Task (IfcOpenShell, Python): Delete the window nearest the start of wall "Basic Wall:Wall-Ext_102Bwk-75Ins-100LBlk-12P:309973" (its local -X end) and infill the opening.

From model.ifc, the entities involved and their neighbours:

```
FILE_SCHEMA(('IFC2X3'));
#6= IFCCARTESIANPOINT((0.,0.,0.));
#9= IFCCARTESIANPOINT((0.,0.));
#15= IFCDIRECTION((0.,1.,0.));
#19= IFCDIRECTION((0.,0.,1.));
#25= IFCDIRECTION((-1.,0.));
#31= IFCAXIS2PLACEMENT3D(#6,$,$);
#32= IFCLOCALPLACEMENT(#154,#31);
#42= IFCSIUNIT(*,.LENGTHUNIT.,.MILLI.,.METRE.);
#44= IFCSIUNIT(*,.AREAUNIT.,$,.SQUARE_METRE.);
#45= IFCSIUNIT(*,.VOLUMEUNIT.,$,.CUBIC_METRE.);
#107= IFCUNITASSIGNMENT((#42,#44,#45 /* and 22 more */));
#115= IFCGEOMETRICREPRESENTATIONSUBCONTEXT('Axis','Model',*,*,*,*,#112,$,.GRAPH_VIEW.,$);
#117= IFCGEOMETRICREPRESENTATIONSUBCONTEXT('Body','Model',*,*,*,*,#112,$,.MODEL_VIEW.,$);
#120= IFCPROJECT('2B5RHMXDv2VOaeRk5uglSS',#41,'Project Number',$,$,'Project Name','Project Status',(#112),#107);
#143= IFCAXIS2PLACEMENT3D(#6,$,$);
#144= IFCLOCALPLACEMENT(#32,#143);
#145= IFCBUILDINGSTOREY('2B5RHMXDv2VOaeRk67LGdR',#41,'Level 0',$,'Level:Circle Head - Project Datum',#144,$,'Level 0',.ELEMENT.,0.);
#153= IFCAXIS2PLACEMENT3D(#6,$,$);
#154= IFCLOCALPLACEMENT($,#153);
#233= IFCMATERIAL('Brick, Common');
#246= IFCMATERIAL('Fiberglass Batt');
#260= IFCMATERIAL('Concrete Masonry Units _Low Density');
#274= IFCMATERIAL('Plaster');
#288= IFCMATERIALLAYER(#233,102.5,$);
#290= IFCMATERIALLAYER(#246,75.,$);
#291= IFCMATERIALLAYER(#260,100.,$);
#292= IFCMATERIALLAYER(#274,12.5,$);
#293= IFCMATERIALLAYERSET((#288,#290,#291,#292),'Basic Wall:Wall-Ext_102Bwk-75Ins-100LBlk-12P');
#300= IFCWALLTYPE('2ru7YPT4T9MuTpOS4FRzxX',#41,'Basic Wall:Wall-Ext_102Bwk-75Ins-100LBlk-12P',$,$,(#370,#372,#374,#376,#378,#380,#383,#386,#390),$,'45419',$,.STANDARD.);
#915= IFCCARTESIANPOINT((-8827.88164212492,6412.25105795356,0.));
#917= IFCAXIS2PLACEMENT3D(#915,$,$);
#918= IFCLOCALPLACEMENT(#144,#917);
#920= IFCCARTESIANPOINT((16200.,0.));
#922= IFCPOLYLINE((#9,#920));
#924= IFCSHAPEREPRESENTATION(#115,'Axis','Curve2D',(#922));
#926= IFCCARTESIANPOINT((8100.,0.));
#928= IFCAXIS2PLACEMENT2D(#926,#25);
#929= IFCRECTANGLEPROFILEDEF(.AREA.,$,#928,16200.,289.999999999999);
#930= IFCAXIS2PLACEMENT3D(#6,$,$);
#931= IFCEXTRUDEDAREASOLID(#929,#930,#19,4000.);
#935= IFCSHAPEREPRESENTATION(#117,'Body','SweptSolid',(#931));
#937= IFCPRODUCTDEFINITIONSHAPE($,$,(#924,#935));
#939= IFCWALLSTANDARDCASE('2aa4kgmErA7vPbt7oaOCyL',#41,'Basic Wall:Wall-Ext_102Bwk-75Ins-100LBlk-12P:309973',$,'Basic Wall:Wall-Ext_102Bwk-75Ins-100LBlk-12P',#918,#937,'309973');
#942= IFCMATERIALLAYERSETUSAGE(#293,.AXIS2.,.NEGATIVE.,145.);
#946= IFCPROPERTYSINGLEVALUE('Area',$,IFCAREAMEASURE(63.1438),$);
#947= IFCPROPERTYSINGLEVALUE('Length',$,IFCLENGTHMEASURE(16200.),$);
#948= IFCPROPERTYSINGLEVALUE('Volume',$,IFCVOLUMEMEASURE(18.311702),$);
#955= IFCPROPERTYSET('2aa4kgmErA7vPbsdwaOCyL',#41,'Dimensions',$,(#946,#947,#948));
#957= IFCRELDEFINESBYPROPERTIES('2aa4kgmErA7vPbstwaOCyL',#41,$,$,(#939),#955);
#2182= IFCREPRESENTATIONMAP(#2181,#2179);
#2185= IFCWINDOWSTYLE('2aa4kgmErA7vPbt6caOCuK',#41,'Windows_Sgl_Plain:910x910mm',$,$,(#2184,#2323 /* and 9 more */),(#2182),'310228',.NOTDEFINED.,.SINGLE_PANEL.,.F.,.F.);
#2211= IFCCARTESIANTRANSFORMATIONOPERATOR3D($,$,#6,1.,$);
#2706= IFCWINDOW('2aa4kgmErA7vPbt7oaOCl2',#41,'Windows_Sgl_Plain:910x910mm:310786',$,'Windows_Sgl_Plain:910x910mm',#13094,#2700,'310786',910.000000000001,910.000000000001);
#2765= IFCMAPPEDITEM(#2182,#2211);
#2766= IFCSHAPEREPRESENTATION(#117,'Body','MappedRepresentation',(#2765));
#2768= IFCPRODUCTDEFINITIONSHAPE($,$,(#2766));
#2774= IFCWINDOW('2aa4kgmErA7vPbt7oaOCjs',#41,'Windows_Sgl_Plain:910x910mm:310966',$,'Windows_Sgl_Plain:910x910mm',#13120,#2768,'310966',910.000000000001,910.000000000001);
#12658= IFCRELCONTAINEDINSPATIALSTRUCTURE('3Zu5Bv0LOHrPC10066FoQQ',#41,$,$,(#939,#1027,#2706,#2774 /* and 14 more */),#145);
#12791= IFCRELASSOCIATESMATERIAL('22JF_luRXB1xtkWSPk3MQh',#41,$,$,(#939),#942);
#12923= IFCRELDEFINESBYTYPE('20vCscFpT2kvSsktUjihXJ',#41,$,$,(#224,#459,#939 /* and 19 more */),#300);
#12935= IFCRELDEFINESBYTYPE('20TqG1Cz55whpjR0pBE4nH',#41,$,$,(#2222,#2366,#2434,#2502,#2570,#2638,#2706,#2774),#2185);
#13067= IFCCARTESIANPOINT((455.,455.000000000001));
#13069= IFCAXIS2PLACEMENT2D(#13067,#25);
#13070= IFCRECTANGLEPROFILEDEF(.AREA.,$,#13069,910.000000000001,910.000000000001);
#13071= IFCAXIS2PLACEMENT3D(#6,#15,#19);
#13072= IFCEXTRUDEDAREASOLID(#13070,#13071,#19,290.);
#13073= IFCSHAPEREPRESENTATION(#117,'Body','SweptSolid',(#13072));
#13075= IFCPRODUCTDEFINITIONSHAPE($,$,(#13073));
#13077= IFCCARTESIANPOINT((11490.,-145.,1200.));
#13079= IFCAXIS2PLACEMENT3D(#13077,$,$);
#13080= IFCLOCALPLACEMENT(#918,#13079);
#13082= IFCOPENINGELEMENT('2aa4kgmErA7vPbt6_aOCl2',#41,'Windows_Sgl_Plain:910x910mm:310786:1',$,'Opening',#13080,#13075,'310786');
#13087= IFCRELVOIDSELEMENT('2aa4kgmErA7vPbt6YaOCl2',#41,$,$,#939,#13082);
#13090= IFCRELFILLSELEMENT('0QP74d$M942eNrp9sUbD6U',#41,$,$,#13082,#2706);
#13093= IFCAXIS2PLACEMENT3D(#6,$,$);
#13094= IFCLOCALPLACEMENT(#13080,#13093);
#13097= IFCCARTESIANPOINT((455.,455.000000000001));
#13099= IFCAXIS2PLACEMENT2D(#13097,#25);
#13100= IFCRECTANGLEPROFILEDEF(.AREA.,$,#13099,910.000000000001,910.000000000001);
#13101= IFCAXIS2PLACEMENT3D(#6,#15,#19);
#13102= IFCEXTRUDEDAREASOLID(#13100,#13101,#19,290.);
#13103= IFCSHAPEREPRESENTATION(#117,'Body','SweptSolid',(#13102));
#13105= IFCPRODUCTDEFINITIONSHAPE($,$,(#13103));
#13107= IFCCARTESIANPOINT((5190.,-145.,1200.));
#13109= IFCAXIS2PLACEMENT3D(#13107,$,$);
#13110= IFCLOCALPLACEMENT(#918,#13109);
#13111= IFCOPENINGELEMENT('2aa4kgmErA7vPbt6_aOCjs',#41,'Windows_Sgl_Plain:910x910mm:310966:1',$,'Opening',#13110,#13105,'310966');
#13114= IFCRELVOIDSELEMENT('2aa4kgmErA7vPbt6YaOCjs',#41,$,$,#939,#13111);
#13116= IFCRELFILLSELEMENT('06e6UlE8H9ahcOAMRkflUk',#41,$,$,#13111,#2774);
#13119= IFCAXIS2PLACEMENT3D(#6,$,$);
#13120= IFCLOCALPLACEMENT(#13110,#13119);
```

```python
import ifcopenshell
import ifcopenshell.api.feature
import ifcopenshell.api.pset
import ifcopenshell.api.root
import ifcopenshell.geom
import ifcopenshell.util.element
import ifcopenshell.util.shape
import ifcopenshell.util.unit

model = ifcopenshell.open("model.ifc")
area_scale = ifcopenshell.util.unit.calculate_unit_scale(model, "AREAUNIT")
volume_scale = ifcopenshell.util.unit.calculate_unit_scale(model, "VOLUMEUNIT")
settings = ifcopenshell.geom.settings()


def volume(element):
    """Net volume in cubic metres, openings subtracted."""
    shape = ifcopenshell.geom.create_shape(settings, element)
    return ifcopenshell.util.shape.get_volume(shape.geometry)


window = model.by_id(2774)
opening = window.FillsVoids[0].RelatingOpeningElement
wall = opening.VoidsElements[0].RelatingBuildingElement
before = volume(wall)

ifcopenshell.api.root.remove_product(model, product=window)
ifcopenshell.api.feature.remove_feature(model, feature=opening)

after = volume(wall)
thickness = 0.29  # wall thickness in metres

# Update the wall's stored quantities.
pset = model.by_id(ifcopenshell.util.element.get_pset(wall, "Dimensions", should_inherit=False)["id"])
ifcopenshell.api.pset.edit_pset(model, pset=pset, properties={
    "Area": model.create_entity("IfcAreaMeasure", after / thickness / area_scale),
    "Volume": model.create_entity("IfcVolumeMeasure", after / volume_scale),
})

print(f"wall volume {before:.3f} -> {after:.3f} m3")

model.write("model_updated.ifc")
```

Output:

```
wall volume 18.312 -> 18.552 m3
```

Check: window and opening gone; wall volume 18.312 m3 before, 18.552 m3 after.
